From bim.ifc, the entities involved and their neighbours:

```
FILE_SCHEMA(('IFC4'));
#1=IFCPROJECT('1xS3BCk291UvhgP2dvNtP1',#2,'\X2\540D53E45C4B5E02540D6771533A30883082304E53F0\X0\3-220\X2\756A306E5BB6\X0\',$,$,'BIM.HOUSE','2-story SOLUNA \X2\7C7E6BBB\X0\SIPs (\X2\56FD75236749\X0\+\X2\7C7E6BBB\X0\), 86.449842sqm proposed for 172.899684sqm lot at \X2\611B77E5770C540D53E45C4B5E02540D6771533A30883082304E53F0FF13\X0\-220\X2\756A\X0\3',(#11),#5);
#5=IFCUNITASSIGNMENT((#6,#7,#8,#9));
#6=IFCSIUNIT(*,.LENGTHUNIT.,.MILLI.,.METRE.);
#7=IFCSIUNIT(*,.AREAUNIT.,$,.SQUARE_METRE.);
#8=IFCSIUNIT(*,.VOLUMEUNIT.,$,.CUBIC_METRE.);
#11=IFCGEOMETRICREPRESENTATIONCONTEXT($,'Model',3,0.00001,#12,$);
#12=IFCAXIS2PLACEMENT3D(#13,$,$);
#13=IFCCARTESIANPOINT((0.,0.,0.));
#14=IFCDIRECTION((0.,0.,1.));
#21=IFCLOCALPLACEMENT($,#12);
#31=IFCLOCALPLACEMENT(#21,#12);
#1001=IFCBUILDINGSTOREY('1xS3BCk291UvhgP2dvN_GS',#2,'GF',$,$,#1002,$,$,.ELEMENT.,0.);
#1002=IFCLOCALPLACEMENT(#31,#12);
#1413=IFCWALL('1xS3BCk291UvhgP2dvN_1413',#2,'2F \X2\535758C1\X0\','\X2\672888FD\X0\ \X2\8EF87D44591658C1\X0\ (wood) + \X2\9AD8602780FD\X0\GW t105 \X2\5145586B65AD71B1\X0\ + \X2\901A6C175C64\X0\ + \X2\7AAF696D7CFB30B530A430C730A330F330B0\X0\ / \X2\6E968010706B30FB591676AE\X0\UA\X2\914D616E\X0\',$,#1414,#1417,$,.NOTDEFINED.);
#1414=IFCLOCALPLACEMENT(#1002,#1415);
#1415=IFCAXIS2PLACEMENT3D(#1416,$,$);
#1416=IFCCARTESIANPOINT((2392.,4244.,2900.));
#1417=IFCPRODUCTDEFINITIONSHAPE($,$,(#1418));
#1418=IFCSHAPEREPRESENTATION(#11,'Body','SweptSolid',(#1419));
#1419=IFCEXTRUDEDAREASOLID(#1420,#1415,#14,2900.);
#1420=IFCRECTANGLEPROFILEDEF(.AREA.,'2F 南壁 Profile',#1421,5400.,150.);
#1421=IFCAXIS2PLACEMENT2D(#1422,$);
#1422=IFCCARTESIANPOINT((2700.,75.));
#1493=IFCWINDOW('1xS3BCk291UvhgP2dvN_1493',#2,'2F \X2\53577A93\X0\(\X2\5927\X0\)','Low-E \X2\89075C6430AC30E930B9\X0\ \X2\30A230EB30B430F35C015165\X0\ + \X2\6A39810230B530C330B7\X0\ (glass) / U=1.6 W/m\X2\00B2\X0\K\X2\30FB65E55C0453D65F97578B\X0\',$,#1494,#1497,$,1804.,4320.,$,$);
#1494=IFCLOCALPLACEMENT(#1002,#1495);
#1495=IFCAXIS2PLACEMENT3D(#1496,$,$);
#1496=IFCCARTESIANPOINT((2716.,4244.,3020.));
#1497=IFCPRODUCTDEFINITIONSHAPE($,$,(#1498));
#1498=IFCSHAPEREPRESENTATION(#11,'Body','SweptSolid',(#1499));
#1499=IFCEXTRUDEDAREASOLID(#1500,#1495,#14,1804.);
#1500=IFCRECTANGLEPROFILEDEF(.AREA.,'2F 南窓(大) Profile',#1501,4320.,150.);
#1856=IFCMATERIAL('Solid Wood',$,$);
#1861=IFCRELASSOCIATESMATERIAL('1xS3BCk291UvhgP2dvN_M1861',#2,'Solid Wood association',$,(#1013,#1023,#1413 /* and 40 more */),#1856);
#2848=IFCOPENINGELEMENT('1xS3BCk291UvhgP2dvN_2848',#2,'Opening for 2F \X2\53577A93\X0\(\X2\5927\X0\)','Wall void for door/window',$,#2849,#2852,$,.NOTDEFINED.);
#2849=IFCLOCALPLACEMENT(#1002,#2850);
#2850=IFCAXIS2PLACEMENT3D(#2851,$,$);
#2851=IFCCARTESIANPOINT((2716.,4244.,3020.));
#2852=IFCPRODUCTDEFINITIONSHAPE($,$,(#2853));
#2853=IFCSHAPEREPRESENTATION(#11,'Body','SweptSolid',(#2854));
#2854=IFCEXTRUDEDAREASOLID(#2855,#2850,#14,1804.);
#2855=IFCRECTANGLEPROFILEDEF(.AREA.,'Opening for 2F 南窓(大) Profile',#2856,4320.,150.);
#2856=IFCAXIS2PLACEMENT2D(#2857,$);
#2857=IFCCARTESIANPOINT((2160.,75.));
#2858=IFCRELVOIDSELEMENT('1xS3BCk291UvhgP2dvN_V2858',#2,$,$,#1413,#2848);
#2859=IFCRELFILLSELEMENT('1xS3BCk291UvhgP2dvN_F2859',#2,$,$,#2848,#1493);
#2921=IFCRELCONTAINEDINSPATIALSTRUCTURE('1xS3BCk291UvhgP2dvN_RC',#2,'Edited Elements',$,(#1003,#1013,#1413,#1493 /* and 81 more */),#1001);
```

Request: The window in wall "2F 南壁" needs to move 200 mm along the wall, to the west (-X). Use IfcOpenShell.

```python
import ifcopenshell
import ifcopenshell.api.geometry
import ifcopenshell.util.placement

model = ifcopenshell.open("bim.ifc")

window = model.by_guid("1xS3BCk291UvhgP2dvN_1493")
opening = window.FillsVoids[0].RelatingOpeningElement
wall = opening.VoidsElements[0].RelatingBuildingElement

wall_matrix = ifcopenshell.util.placement.get_local_placement(wall.ObjectPlacement)
shift = wall_matrix[:3, 0] * -200.0
before = ifcopenshell.util.placement.get_local_placement(window.ObjectPlacement)[:3, 3].copy()

# The window is not placed relative to its opening, so move both.
for product in (opening, window):
    matrix = ifcopenshell.util.placement.get_local_placement(product.ObjectPlacement)
    matrix[:3, 3] += shift
    ifcopenshell.api.geometry.edit_object_placement(model, product=product, matrix=matrix, is_si=False)

after = ifcopenshell.util.placement.get_local_placement(window.ObjectPlacement)[:3, 3]
print("window moved by", (after - before).round(3) + 0.0)

model.write("bim_rev.ifc")
```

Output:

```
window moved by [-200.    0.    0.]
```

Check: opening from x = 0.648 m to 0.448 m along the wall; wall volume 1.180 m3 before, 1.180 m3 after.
